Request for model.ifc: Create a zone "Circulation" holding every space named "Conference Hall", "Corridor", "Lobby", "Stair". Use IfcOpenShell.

First a look at what the model holds.

```python
import ifcopenshell

model = ifcopenshell.open("model.ifc")
print(model.schema)
seen = {}
for space in model.by_type("IfcSpace"):
    seen[space.LongName] = seen.get(space.LongName, 0) + 1
for name, count in sorted(seen.items(), key=str):
    print(count, "x", name)
print("zones:", [z.Name for z in model.by_type("IfcZone")][:20])
```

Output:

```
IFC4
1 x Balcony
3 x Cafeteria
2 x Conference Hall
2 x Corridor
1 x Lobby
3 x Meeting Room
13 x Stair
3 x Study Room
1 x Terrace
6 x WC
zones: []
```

```python
import ifcopenshell
import ifcopenshell.api.group
import ifcopenshell.api.root

model = ifcopenshell.open("model.ifc")

names = {"Conference Hall", "Corridor", "Lobby", "Stair"}
spaces = [s for s in model.by_type("IfcSpace") if s.LongName in names]

zone = ifcopenshell.api.root.create_entity(model, ifc_class="IfcZone", name="Circulation")
ifcopenshell.api.group.assign_group(model, products=spaces, group=zone)
print(len(spaces), "spaces in", zone.Name)

model.write("model_updated.ifc")
```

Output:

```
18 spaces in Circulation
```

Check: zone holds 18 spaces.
